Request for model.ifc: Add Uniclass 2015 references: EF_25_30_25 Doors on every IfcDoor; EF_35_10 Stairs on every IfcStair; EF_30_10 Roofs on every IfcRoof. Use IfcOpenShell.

First a look at what the model holds.

```python
import ifcopenshell

model = ifcopenshell.open("model.ifc")
print(model.schema)
print("classifications:", [c.Name for c in model.by_type("IfcClassification")])
for ifc_class in ("IfcDoor", "IfcRoof", "IfcStair", "IfcWall", "IfcWindow"):
    print(ifc_class, len(model.by_type(ifc_class)))
```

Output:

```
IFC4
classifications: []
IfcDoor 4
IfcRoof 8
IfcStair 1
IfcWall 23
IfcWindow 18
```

```python
import ifcopenshell
import ifcopenshell.api.classification

model = ifcopenshell.open("model.ifc")

system = ifcopenshell.api.classification.add_classification(model, classification="Uniclass 2015")

codes = {
    "IfcDoor": ("EF_25_30_25", "Doors"),
    "IfcStair": ("EF_35_10", "Stairs"),
    "IfcRoof": ("EF_30_10", "Roofs"),
}
for ifc_class, (code, name) in codes.items():
    products = model.by_type(ifc_class)
    ifcopenshell.api.classification.add_reference(
        model, products=products, classification=system, identification=code, name=name
    )
    print(code, len(products))

model.write("model-out.ifc")
```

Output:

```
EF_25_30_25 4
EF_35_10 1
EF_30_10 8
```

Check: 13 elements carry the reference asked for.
